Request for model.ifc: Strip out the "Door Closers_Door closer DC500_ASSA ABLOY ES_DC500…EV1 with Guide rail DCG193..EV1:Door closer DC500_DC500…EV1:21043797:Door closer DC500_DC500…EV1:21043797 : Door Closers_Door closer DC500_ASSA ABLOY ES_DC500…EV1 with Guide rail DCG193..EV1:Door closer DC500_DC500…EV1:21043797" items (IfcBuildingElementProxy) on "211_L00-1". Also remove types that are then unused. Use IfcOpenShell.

First a look at what the model holds.

```python
import ifcopenshell
import ifcopenshell.util.element

model = ifcopenshell.open("model.ifc")
print(model.schema)
storey = next(s for s in model.by_type("IfcBuildingStorey") if s.Name == "211_L00-1")
proxies = [e for e in ifcopenshell.util.element.get_decomposition(storey) if e.is_a("IfcBuildingElementProxy")]
seen = {}
for e in proxies:
    element_type = ifcopenshell.util.element.get_type(e)
    name = element_type.Name if element_type not in (None, e) else None
    seen[name] = seen.get(name, 0) + 1
for name, count in sorted(seen.items(), key=str):
    print(count, "x", name)
```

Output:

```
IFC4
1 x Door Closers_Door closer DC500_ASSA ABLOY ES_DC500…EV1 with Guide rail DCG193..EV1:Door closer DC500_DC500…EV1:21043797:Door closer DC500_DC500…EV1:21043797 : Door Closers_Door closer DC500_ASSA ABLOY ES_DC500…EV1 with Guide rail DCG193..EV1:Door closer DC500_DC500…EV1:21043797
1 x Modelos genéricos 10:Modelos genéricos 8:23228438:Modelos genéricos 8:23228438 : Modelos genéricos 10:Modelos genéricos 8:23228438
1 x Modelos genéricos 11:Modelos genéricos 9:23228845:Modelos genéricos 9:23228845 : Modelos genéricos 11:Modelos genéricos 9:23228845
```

```python
import ifcopenshell
import ifcopenshell.api.root
import ifcopenshell.util.element

model = ifcopenshell.open("model.ifc")

storey = next(s for s in model.by_type("IfcBuildingStorey") if s.Name == "211_L00-1")
proxies = [e for e in ifcopenshell.util.element.get_decomposition(storey) if e.is_a("IfcBuildingElementProxy")]
targets = [e for e in proxies if (t := ifcopenshell.util.element.get_type(e)) not in (None, e) and t.Name == "Door Closers_Door closer DC500_ASSA ABLOY ES_DC500…EV1 with Guide rail DCG193..EV1:Door closer DC500_DC500…EV1:21043797:Door closer DC500_DC500…EV1:21043797 : Door Closers_Door closer DC500_ASSA ABLOY ES_DC500…EV1 with Guide rail DCG193..EV1:Door closer DC500_DC500…EV1:21043797"]
types = {ifcopenshell.util.element.get_type(e) for e in targets} - {None, *targets}

for e in targets:
    ifcopenshell.api.root.remove_product(model, product=e)
print(len(targets), "removed")

unused = [t for t in types if not ifcopenshell.util.element.get_types(t)]
for t in unused:
    ifcopenshell.api.root.remove_product(model, product=t)
print(len(unused), "unused types removed")

model.write("model_v2.ifc")
```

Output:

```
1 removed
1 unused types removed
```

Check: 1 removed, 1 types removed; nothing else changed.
